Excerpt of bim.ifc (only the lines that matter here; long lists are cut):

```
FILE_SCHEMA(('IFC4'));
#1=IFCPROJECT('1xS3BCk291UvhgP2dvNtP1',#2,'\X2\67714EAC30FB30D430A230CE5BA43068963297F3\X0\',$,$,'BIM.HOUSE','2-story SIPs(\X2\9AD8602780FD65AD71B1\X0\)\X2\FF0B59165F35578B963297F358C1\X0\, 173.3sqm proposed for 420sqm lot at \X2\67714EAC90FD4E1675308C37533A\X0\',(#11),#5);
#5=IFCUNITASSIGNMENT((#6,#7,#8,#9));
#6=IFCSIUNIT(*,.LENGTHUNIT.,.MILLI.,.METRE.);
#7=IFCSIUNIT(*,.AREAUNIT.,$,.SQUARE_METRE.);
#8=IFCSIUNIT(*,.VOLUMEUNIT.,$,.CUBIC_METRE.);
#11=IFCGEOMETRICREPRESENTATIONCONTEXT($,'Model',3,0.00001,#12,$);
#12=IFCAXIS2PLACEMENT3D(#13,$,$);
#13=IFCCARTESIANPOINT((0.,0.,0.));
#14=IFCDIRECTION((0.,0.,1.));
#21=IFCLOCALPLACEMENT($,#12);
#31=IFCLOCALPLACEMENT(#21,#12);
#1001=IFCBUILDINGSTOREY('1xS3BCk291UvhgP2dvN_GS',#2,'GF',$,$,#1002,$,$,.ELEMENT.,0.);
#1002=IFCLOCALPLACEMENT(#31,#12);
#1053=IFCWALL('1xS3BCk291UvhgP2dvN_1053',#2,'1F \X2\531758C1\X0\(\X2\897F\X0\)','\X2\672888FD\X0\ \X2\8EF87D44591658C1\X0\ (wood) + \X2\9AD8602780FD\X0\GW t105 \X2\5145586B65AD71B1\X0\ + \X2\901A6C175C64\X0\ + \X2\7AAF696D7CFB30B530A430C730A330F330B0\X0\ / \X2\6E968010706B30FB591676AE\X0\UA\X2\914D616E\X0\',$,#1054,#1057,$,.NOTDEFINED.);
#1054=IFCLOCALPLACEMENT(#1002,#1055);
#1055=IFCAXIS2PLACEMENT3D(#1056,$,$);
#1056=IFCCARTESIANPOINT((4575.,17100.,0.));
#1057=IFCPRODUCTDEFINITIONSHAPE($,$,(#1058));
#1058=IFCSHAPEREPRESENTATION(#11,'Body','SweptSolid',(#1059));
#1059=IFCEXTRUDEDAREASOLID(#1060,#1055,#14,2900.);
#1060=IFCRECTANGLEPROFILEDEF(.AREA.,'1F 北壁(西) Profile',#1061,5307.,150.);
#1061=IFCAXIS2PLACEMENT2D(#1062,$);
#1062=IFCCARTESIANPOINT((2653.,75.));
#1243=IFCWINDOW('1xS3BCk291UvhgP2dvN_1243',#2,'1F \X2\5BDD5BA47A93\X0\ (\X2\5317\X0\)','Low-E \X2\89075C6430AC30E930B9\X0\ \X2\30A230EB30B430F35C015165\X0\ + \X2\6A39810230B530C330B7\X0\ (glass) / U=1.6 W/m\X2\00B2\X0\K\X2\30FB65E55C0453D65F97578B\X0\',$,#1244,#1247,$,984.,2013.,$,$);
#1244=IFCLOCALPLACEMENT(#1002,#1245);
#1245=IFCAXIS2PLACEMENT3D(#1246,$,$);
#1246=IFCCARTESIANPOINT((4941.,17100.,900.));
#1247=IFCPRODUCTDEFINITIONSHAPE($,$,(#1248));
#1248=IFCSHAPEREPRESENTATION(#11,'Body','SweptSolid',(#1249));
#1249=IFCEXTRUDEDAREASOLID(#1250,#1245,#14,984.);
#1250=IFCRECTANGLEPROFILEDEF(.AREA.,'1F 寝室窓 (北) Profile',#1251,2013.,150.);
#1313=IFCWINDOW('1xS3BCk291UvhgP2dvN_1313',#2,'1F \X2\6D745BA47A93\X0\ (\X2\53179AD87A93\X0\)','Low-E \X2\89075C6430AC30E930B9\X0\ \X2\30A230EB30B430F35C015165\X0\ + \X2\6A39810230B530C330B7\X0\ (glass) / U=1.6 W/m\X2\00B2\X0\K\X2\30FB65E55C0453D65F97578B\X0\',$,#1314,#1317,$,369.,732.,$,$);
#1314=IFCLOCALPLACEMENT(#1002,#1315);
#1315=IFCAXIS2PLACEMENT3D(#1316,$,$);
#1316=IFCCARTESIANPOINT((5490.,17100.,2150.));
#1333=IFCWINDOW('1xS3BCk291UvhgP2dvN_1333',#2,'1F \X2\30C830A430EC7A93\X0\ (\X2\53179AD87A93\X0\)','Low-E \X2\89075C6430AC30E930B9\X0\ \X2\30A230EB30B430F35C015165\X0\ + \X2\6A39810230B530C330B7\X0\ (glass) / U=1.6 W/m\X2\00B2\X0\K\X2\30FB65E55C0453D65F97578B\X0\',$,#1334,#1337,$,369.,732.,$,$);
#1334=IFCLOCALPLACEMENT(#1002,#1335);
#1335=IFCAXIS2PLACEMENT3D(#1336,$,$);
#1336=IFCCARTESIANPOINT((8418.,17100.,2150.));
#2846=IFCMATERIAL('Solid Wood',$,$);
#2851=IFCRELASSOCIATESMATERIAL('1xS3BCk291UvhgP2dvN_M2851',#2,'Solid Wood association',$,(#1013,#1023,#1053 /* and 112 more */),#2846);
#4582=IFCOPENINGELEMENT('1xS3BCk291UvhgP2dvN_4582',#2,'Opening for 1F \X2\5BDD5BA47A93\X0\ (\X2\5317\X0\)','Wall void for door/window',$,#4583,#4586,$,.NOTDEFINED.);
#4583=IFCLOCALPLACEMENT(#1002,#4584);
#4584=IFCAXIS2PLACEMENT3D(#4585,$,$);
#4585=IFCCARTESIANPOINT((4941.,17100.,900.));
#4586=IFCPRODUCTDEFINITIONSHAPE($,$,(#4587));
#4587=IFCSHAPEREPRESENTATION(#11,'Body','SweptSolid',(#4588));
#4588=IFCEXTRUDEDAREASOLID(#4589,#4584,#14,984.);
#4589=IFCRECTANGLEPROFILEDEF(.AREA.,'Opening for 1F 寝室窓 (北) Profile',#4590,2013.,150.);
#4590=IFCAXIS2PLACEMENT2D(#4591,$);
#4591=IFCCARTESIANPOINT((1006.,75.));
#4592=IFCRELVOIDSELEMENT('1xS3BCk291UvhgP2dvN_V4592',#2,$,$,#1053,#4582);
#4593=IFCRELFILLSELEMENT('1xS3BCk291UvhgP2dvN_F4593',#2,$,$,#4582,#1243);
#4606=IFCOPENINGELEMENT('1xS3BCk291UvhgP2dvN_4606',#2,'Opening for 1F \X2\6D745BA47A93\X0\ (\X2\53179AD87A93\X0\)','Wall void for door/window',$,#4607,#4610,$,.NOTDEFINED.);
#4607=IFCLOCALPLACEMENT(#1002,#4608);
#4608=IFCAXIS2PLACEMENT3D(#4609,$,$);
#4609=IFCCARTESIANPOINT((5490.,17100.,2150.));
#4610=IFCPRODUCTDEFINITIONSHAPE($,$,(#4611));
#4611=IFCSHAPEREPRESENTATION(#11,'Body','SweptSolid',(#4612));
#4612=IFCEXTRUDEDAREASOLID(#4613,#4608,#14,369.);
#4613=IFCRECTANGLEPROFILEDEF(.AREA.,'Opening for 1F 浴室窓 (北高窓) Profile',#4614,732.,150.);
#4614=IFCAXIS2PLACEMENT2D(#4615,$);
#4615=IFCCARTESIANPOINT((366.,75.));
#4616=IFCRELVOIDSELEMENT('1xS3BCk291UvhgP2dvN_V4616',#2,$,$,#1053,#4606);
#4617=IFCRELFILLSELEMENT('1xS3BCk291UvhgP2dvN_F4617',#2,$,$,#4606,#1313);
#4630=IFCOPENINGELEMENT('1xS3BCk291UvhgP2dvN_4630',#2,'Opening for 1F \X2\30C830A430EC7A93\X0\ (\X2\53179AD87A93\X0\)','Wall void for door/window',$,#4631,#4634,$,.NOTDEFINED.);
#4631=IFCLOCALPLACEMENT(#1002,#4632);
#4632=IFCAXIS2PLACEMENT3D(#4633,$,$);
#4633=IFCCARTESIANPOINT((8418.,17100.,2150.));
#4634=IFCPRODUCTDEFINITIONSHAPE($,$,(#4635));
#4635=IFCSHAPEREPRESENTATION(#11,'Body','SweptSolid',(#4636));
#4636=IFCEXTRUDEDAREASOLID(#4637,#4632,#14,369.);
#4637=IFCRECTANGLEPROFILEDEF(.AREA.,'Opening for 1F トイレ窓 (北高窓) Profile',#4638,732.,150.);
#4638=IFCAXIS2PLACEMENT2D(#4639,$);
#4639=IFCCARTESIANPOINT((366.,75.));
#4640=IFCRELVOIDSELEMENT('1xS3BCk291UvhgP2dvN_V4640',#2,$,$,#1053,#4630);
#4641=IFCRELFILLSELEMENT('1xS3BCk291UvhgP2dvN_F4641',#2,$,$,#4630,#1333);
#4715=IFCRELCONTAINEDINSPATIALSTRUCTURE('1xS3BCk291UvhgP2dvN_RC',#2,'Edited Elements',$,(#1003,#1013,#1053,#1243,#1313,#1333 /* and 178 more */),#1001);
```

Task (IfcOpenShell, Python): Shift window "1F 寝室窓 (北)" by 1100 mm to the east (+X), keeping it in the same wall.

```python
import ifcopenshell
import ifcopenshell.api.geometry
import ifcopenshell.util.placement
import ifcopenshell.util.unit

model = ifcopenshell.open("bim.ifc")
unit_scale = ifcopenshell.util.unit.calculate_unit_scale(model)

window = model.by_guid("1xS3BCk291UvhgP2dvN_1243")
opening = window.FillsVoids[0].RelatingOpeningElement
wall = opening.VoidsElements[0].RelatingBuildingElement

wall_matrix = ifcopenshell.util.placement.get_local_placement(wall.ObjectPlacement)
shift = wall_matrix[:3, 0] * 1.1 / unit_scale
before = ifcopenshell.util.placement.get_local_placement(window.ObjectPlacement)[:3, 3].copy()

# The window is not placed relative to its opening, so move both.
for product in (opening, window):
    matrix = ifcopenshell.util.placement.get_local_placement(product.ObjectPlacement)
    matrix[:3, 3] += shift
    ifcopenshell.api.geometry.edit_object_placement(model, product=product, matrix=matrix, is_si=False)

after = ifcopenshell.util.placement.get_local_placement(window.ObjectPlacement)[:3, 3]
print("window moved by", (after - before).round(3) + 0.0)

model.write("bim-out.ifc")
```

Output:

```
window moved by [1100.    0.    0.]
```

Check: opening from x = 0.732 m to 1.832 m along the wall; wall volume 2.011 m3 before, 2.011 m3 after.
